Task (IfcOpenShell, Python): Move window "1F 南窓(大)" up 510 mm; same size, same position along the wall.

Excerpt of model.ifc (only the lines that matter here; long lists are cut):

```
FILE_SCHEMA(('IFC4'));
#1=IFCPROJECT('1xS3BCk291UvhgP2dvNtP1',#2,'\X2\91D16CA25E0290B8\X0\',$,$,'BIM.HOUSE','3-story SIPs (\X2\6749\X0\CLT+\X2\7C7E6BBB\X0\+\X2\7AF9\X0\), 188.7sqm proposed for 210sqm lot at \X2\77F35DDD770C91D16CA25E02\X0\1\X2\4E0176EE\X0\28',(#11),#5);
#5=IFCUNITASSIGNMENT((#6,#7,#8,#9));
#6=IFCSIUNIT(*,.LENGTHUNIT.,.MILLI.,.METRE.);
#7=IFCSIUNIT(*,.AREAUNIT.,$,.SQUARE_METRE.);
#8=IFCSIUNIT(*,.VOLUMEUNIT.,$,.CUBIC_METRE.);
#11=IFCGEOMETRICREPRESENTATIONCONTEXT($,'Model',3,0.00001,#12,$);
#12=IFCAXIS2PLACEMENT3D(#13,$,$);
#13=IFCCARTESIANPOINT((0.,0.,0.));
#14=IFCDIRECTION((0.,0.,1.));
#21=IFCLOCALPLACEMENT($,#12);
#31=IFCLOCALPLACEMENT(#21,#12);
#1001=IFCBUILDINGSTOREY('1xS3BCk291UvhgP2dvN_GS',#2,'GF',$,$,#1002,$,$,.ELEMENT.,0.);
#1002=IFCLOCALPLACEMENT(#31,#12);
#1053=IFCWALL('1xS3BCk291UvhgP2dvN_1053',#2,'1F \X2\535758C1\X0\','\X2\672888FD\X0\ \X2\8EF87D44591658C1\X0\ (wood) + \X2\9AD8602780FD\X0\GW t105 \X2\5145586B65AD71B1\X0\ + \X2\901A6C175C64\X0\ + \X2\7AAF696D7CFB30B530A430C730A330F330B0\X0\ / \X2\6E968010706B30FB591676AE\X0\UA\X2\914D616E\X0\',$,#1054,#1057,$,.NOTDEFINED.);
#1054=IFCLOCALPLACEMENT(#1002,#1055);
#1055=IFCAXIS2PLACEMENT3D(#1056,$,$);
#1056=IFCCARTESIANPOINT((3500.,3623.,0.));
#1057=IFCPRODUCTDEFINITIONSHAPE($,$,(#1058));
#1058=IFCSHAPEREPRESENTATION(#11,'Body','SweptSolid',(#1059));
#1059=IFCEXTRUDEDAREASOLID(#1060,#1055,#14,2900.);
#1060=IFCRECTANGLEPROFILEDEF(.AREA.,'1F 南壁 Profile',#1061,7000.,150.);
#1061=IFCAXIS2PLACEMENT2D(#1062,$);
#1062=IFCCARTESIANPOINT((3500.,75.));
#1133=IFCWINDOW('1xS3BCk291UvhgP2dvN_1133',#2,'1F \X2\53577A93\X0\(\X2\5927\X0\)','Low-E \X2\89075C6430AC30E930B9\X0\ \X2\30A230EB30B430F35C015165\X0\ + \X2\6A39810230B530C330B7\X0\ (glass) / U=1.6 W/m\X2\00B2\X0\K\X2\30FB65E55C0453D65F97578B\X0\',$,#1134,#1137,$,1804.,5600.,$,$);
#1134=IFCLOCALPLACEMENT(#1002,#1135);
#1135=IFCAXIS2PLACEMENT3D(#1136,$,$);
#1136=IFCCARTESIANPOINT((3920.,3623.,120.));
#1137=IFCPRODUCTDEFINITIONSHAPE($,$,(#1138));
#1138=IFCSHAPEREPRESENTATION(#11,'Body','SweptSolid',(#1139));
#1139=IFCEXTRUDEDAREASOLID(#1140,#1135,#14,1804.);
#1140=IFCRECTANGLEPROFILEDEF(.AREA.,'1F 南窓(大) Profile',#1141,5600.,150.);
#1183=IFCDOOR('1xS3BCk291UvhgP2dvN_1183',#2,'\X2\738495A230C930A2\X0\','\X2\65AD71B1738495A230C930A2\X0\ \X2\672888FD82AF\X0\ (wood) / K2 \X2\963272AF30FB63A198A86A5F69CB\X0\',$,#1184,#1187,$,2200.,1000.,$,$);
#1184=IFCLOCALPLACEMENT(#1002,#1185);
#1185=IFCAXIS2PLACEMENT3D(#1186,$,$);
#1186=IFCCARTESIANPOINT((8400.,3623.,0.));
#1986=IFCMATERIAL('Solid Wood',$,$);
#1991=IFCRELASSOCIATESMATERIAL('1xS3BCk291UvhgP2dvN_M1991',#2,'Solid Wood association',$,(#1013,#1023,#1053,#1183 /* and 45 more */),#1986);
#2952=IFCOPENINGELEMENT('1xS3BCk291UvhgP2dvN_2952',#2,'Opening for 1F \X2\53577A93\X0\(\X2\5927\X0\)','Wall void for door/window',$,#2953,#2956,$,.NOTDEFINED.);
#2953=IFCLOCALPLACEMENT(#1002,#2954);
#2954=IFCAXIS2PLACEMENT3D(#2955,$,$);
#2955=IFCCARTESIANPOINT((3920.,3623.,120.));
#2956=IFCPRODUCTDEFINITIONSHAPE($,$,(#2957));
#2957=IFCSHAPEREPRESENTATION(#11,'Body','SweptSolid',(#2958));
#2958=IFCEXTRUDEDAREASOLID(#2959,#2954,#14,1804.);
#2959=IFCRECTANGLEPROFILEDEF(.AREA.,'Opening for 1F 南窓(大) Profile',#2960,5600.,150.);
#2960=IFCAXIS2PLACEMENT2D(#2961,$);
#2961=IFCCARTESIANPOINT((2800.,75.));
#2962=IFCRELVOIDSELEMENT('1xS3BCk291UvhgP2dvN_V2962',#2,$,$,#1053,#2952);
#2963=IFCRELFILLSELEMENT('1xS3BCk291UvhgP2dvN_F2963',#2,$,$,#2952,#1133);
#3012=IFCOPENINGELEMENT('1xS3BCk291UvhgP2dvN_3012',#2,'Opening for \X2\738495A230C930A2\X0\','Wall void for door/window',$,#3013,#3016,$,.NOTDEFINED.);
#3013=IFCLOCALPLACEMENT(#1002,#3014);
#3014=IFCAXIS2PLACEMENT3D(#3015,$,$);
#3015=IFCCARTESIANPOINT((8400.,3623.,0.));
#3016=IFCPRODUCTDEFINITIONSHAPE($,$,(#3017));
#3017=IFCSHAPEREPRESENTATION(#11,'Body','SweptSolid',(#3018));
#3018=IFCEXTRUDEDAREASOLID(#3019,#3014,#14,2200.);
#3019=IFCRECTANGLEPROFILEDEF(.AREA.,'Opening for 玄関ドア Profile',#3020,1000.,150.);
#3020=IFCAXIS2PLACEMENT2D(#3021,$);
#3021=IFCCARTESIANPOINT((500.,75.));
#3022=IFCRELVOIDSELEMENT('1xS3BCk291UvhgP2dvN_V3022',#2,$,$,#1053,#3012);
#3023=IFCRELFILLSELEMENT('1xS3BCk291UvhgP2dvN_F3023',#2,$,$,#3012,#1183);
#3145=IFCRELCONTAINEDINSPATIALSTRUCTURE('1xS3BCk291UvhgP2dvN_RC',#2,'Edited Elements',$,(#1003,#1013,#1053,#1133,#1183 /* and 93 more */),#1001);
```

```python
import numpy as np
import ifcopenshell
import ifcopenshell.api.geometry
import ifcopenshell.util.placement
import ifcopenshell.util.unit

model = ifcopenshell.open("model.ifc")
unit_scale = ifcopenshell.util.unit.calculate_unit_scale(model)

window = model.by_id(1133)
opening = window.FillsVoids[0].RelatingOpeningElement
dz = 0.51 / unit_scale

shift = np.array([0.0, 0.0, dz])
# The window is not placed relative to its opening, so move both.
for product in (opening, window):
    matrix = ifcopenshell.util.placement.get_local_placement(product.ObjectPlacement)
    matrix[:3, 3] += shift
    ifcopenshell.api.geometry.edit_object_placement(model, product=product, matrix=matrix, is_si=False)

print(f"moved by {dz * unit_scale:+.3f} m")

model.write("model_edited.ifc")
```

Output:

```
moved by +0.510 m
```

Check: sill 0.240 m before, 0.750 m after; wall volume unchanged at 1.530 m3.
